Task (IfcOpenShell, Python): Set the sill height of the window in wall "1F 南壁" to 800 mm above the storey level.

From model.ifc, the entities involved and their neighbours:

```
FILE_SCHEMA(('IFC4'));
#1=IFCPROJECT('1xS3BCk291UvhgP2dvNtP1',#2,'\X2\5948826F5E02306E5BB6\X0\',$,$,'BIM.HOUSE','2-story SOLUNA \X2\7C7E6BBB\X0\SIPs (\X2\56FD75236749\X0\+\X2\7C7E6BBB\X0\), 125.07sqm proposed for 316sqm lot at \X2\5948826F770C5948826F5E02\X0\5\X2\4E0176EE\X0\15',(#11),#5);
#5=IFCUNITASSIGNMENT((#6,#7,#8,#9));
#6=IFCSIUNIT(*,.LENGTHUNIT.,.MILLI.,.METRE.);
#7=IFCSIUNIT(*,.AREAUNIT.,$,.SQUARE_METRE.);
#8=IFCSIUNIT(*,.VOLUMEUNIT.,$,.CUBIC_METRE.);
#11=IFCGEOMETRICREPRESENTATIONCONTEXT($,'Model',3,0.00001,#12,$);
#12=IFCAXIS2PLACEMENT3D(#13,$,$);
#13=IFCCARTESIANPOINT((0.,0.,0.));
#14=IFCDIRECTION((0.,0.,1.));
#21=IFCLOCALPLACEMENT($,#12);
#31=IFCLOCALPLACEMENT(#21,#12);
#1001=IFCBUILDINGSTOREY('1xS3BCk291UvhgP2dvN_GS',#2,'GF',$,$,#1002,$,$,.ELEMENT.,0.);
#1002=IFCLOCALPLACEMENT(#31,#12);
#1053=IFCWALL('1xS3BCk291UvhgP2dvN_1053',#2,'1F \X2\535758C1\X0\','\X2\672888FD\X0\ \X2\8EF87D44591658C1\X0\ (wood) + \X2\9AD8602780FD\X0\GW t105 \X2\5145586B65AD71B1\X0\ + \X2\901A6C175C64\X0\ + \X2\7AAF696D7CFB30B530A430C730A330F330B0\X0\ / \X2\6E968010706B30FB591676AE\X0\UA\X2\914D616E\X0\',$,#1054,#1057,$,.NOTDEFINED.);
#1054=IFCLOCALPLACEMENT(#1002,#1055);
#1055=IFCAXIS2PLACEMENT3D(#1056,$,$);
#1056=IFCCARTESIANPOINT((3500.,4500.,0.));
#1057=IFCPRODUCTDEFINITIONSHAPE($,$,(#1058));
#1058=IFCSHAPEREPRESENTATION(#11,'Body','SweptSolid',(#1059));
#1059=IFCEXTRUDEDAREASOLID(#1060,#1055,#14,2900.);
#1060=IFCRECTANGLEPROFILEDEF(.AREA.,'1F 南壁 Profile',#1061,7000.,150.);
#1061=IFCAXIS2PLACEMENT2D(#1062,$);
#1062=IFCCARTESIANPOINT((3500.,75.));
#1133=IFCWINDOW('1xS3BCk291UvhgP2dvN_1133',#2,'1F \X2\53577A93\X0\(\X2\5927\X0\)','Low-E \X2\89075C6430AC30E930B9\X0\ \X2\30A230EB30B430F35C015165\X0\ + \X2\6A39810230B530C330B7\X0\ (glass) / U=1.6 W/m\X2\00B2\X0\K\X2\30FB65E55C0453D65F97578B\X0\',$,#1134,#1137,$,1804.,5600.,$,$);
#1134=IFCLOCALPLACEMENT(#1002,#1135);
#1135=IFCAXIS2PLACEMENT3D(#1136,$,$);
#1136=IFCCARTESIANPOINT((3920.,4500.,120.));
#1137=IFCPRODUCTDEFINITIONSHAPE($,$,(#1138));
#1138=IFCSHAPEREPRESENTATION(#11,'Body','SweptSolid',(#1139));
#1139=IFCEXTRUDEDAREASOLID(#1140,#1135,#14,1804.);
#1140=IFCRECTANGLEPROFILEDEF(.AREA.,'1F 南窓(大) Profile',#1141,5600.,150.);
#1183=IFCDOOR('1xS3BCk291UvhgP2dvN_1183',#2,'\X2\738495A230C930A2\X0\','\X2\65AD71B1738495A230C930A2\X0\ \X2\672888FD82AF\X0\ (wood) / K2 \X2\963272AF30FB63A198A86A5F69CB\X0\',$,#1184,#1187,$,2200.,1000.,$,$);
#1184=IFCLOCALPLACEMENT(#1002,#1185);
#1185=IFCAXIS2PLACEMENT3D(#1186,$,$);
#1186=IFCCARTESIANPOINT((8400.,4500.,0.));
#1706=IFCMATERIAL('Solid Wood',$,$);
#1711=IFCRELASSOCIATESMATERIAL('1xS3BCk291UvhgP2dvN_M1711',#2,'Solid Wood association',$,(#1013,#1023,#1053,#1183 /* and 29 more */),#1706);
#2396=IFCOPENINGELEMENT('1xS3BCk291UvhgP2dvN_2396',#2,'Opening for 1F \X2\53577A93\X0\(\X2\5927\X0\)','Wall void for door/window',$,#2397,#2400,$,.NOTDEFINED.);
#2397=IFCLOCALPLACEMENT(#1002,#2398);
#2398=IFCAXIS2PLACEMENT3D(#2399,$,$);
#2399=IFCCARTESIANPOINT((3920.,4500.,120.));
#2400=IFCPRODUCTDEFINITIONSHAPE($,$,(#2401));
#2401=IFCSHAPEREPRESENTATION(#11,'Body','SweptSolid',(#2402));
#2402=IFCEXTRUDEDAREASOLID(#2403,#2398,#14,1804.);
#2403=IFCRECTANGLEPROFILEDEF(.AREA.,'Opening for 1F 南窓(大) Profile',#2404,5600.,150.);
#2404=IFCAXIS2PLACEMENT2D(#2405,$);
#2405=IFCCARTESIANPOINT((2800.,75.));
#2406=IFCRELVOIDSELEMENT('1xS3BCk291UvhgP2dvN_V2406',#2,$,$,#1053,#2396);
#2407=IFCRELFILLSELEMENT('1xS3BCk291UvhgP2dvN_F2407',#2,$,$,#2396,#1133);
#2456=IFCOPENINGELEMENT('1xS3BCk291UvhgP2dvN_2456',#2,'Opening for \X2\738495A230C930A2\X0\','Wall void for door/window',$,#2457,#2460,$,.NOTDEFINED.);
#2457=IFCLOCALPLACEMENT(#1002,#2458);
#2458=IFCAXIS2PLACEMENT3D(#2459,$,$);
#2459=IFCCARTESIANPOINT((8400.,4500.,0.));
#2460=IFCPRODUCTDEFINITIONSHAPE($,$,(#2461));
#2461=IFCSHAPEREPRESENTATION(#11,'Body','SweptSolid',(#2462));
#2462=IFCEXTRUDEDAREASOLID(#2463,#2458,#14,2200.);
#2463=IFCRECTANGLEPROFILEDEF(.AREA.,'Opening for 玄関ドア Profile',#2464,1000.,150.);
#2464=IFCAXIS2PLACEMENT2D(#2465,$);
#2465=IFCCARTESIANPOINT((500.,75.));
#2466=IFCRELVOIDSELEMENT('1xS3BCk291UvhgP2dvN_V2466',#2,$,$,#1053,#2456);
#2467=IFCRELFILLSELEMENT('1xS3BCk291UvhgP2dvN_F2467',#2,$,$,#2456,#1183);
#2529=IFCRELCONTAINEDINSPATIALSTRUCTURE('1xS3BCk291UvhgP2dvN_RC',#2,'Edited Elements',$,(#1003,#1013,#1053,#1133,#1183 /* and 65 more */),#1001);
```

```python
import numpy as np
import ifcopenshell
import ifcopenshell.api.geometry
import ifcopenshell.geom
import ifcopenshell.util.element
import ifcopenshell.util.placement
import ifcopenshell.util.shape
import ifcopenshell.util.unit

model = ifcopenshell.open("model.ifc")
unit_scale = ifcopenshell.util.unit.calculate_unit_scale(model)

window = model.by_id(1133)
opening = window.FillsVoids[0].RelatingOpeningElement
storey = ifcopenshell.util.element.get_container(window, ifc_class="IfcBuildingStorey")
level = ifcopenshell.util.placement.get_local_placement(storey.ObjectPlacement)[2, 3]

# The opening's origin need not be at the sill, so measure its lowest point.
shape = ifcopenshell.geom.create_shape(ifcopenshell.geom.settings(), opening)
bottom = ifcopenshell.util.shape.get_shape_bottom_elevation(shape, shape.geometry) / unit_scale
dz = level + 800.0 - bottom

shift = np.array([0.0, 0.0, dz])
# The window is not placed relative to its opening, so move both.
for product in (opening, window):
    matrix = ifcopenshell.util.placement.get_local_placement(product.ObjectPlacement)
    matrix[:3, 3] += shift
    ifcopenshell.api.geometry.edit_object_placement(model, product=product, matrix=matrix, is_si=False)

print(f"moved by {dz * unit_scale:+.3f} m")

model.write("model_v2.ifc")
```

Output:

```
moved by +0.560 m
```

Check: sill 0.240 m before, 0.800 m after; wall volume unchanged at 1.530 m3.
